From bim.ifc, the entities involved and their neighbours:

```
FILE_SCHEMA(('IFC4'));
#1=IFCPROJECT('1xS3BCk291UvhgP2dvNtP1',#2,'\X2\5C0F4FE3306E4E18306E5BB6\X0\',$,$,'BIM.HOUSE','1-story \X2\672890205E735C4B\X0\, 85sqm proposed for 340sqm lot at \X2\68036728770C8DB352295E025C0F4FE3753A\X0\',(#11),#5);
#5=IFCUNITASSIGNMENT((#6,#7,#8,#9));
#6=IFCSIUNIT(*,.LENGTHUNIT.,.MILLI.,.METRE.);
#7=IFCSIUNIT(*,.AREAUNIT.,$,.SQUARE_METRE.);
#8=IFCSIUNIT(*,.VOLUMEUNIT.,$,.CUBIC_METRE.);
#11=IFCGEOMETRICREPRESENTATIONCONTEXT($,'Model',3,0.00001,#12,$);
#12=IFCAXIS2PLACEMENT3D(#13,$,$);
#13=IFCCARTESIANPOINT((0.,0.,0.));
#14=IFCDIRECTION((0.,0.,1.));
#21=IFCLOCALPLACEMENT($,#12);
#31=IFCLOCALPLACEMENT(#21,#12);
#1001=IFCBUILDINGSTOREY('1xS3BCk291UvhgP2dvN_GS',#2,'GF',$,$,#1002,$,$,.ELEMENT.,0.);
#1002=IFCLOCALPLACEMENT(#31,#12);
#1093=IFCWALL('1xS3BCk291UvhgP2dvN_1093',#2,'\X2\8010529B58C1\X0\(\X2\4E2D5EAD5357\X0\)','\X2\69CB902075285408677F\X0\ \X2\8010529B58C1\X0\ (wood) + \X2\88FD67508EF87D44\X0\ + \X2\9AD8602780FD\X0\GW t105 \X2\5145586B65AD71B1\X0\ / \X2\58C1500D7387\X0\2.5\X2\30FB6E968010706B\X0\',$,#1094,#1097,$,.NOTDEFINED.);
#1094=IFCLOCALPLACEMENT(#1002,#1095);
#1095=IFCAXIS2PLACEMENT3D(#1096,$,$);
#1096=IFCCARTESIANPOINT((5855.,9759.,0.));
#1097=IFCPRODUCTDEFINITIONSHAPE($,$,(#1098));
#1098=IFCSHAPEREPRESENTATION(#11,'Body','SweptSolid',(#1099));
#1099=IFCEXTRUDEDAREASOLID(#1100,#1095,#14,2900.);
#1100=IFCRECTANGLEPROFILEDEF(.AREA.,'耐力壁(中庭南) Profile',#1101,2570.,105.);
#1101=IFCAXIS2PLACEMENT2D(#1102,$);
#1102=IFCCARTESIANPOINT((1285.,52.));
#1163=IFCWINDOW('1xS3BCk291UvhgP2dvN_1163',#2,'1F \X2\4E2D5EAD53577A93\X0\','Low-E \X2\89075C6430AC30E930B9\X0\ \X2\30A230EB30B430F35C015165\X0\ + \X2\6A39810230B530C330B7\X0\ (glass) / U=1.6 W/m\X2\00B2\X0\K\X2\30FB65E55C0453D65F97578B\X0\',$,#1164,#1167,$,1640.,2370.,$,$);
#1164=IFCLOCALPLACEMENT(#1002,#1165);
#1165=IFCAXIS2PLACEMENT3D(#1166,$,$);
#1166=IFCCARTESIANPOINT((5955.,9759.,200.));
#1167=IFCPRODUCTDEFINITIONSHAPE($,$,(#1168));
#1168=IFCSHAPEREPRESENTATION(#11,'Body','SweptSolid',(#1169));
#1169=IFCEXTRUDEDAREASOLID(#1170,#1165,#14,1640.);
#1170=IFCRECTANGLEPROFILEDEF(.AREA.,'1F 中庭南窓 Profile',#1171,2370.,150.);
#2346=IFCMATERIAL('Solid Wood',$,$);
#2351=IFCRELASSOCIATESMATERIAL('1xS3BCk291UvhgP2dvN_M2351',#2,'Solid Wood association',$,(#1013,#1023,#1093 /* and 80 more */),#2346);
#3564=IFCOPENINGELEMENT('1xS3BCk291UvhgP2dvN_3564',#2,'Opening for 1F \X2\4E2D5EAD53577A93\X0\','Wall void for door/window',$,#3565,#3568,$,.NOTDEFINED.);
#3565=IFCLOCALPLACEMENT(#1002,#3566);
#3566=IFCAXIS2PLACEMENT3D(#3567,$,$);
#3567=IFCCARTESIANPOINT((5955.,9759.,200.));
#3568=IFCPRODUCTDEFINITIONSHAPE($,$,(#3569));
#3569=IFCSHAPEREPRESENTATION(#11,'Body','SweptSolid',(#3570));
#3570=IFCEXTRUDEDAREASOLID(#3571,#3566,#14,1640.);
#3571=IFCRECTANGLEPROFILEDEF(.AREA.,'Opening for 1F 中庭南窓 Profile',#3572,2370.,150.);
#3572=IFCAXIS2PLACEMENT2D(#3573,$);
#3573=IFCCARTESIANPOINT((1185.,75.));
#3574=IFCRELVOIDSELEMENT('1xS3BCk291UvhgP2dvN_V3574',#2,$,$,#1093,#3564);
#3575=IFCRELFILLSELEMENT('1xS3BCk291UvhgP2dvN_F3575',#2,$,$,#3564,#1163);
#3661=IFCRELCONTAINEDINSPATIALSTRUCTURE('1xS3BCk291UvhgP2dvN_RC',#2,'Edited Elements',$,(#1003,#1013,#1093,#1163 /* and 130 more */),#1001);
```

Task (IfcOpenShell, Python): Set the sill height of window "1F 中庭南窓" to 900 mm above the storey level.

```python
import numpy as np
import ifcopenshell
import ifcopenshell.api.geometry
import ifcopenshell.geom
import ifcopenshell.util.element
import ifcopenshell.util.placement
import ifcopenshell.util.shape
import ifcopenshell.util.unit

model = ifcopenshell.open("bim.ifc")
unit_scale = ifcopenshell.util.unit.calculate_unit_scale(model)

window = model.by_id(1163)
opening = window.FillsVoids[0].RelatingOpeningElement
storey = ifcopenshell.util.element.get_container(window, ifc_class="IfcBuildingStorey")
level = ifcopenshell.util.placement.get_local_placement(storey.ObjectPlacement)[2, 3]

# The opening's origin need not be at the sill, so measure its lowest point.
shape = ifcopenshell.geom.create_shape(ifcopenshell.geom.settings(), opening)
bottom = ifcopenshell.util.shape.get_shape_bottom_elevation(shape, shape.geometry) / unit_scale
dz = level + 0.9 / unit_scale - bottom

shift = np.array([0.0, 0.0, dz])
# The window is not placed relative to its opening, so move both.
for product in (opening, window):
    matrix = ifcopenshell.util.placement.get_local_placement(product.ObjectPlacement)
    matrix[:3, 3] += shift
    ifcopenshell.api.geometry.edit_object_placement(model, product=product, matrix=matrix, is_si=False)

print(f"moved by {dz * unit_scale:+.3f} m")

model.write("bim_updated.ifc")
```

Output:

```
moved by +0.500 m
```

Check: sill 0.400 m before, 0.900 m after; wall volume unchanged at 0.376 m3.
